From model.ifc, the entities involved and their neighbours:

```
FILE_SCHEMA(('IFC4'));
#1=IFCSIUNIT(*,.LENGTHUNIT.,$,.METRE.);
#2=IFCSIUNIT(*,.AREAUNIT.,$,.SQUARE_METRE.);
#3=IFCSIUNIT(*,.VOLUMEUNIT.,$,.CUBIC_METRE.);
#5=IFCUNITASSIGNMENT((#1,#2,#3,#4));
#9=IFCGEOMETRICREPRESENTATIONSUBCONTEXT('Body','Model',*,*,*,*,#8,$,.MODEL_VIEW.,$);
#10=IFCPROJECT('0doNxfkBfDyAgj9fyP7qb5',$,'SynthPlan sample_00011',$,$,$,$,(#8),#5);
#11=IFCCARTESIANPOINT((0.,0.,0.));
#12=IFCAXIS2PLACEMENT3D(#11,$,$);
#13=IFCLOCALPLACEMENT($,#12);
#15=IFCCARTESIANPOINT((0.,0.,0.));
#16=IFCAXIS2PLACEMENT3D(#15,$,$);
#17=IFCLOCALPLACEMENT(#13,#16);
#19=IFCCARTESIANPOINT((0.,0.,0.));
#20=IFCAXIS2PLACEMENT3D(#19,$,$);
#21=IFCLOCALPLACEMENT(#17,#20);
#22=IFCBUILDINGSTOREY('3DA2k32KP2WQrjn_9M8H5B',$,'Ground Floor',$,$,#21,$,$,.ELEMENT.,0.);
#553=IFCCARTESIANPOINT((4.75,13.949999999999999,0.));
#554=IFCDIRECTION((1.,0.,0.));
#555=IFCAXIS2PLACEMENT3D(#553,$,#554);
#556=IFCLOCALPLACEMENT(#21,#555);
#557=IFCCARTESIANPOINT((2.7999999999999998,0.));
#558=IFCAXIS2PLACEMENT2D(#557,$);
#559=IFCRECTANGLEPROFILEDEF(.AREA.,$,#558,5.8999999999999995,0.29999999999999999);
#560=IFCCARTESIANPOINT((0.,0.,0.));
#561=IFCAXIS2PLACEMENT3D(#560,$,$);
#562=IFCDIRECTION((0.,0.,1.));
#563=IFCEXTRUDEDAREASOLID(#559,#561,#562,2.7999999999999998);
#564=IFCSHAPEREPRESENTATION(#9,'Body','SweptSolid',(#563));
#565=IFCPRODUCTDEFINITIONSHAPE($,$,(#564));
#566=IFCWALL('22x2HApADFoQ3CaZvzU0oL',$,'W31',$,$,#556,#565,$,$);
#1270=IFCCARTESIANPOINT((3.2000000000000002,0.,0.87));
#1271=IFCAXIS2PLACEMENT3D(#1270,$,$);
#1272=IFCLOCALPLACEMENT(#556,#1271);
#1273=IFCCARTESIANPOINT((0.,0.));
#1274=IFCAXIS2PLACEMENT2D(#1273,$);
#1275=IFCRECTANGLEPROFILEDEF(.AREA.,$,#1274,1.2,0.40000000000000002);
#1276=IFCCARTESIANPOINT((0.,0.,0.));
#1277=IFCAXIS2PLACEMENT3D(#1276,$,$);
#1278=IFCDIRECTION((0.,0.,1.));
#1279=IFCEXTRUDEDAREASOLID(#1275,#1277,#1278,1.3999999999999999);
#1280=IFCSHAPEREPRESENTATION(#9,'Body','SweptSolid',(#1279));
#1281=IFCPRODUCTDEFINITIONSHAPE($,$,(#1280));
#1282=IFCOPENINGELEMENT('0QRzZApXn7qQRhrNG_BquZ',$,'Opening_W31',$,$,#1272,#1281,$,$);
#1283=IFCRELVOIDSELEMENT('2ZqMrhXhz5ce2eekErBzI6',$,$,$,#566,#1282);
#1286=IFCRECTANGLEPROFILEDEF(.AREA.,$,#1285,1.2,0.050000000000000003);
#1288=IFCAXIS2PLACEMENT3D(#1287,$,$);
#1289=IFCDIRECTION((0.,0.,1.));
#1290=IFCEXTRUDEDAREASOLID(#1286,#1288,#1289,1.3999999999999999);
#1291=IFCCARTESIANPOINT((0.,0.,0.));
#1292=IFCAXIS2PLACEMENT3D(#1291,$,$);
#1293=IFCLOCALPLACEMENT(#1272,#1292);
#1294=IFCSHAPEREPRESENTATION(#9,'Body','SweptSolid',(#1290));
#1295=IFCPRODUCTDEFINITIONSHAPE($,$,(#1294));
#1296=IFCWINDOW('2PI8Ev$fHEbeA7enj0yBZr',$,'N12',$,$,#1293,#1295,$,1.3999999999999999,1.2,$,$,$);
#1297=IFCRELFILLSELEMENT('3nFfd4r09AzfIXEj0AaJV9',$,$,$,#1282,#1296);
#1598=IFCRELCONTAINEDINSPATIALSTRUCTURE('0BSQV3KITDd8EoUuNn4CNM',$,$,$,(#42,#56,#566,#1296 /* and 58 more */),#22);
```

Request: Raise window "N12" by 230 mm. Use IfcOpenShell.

```python
import numpy as np
import ifcopenshell
import ifcopenshell.api.geometry
import ifcopenshell.util.placement
import ifcopenshell.util.unit

model = ifcopenshell.open("model.ifc")
unit_scale = ifcopenshell.util.unit.calculate_unit_scale(model)

window = model.by_id(1296)
opening = window.FillsVoids[0].RelatingOpeningElement
dz = 0.23

shift = np.array([0.0, 0.0, dz])
# The window is placed relative to its opening, so it follows when the opening moves.
matrix = ifcopenshell.util.placement.get_local_placement(opening.ObjectPlacement)
matrix[:3, 3] += shift
ifcopenshell.api.geometry.edit_object_placement(
    model, product=opening, matrix=matrix, is_si=False, should_transform_children=True
)

print(f"moved by {dz * unit_scale:+.3f} m")

model.write("model_updated.ifc")
```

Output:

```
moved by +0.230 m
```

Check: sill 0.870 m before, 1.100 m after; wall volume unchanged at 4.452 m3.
